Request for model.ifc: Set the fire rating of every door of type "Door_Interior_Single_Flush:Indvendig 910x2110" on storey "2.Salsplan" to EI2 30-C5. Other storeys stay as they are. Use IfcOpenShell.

First a look at what the model holds.

```python
import ifcopenshell
import ifcopenshell.util.element

model = ifcopenshell.open("model.ifc")
print(model.schema)
storey = next(s for s in model.by_type("IfcBuildingStorey") if s.Name == "2.Salsplan")
doors = [e for e in ifcopenshell.util.element.get_decomposition(storey) if e.is_a("IfcDoor")]
seen = {}
for e in doors:
    element_type = ifcopenshell.util.element.get_type(e)
    key = (element_type.Name if element_type != e and element_type else None, ifcopenshell.util.element.get_pset(e, "Pset_DoorCommon", "FireRating"))
    seen[key] = seen.get(key, 0) + 1
for (name, value), count in sorted(seen.items(), key=str):
    print(count, "x", name, "|", value)
```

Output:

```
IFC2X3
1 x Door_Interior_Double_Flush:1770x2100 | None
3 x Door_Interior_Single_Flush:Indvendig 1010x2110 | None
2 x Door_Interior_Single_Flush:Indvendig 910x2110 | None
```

```python
import ifcopenshell
import ifcopenshell.api.pset
import ifcopenshell.util.element

model = ifcopenshell.open("model.ifc")

storey = next(s for s in model.by_type("IfcBuildingStorey") if s.Name == "2.Salsplan")
doors = [e for e in ifcopenshell.util.element.get_decomposition(storey) if e.is_a("IfcDoor")]

count = 0
for e in doors:
    element_type = ifcopenshell.util.element.get_type(e)
    if element_type in (None, e) or element_type.Name != "Door_Interior_Single_Flush:Indvendig 910x2110":
        continue
    # add_pset returns the element's existing set when there is one.
    pset = ifcopenshell.api.pset.add_pset(model, product=e, name="Pset_DoorCommon")
    ifcopenshell.api.pset.edit_pset(model, pset=pset, properties={"FireRating": "EI2 30-C5"})
    count += 1

print(count, "doors updated")

model.write("model_v2.ifc")
```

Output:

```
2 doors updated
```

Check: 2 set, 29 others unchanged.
